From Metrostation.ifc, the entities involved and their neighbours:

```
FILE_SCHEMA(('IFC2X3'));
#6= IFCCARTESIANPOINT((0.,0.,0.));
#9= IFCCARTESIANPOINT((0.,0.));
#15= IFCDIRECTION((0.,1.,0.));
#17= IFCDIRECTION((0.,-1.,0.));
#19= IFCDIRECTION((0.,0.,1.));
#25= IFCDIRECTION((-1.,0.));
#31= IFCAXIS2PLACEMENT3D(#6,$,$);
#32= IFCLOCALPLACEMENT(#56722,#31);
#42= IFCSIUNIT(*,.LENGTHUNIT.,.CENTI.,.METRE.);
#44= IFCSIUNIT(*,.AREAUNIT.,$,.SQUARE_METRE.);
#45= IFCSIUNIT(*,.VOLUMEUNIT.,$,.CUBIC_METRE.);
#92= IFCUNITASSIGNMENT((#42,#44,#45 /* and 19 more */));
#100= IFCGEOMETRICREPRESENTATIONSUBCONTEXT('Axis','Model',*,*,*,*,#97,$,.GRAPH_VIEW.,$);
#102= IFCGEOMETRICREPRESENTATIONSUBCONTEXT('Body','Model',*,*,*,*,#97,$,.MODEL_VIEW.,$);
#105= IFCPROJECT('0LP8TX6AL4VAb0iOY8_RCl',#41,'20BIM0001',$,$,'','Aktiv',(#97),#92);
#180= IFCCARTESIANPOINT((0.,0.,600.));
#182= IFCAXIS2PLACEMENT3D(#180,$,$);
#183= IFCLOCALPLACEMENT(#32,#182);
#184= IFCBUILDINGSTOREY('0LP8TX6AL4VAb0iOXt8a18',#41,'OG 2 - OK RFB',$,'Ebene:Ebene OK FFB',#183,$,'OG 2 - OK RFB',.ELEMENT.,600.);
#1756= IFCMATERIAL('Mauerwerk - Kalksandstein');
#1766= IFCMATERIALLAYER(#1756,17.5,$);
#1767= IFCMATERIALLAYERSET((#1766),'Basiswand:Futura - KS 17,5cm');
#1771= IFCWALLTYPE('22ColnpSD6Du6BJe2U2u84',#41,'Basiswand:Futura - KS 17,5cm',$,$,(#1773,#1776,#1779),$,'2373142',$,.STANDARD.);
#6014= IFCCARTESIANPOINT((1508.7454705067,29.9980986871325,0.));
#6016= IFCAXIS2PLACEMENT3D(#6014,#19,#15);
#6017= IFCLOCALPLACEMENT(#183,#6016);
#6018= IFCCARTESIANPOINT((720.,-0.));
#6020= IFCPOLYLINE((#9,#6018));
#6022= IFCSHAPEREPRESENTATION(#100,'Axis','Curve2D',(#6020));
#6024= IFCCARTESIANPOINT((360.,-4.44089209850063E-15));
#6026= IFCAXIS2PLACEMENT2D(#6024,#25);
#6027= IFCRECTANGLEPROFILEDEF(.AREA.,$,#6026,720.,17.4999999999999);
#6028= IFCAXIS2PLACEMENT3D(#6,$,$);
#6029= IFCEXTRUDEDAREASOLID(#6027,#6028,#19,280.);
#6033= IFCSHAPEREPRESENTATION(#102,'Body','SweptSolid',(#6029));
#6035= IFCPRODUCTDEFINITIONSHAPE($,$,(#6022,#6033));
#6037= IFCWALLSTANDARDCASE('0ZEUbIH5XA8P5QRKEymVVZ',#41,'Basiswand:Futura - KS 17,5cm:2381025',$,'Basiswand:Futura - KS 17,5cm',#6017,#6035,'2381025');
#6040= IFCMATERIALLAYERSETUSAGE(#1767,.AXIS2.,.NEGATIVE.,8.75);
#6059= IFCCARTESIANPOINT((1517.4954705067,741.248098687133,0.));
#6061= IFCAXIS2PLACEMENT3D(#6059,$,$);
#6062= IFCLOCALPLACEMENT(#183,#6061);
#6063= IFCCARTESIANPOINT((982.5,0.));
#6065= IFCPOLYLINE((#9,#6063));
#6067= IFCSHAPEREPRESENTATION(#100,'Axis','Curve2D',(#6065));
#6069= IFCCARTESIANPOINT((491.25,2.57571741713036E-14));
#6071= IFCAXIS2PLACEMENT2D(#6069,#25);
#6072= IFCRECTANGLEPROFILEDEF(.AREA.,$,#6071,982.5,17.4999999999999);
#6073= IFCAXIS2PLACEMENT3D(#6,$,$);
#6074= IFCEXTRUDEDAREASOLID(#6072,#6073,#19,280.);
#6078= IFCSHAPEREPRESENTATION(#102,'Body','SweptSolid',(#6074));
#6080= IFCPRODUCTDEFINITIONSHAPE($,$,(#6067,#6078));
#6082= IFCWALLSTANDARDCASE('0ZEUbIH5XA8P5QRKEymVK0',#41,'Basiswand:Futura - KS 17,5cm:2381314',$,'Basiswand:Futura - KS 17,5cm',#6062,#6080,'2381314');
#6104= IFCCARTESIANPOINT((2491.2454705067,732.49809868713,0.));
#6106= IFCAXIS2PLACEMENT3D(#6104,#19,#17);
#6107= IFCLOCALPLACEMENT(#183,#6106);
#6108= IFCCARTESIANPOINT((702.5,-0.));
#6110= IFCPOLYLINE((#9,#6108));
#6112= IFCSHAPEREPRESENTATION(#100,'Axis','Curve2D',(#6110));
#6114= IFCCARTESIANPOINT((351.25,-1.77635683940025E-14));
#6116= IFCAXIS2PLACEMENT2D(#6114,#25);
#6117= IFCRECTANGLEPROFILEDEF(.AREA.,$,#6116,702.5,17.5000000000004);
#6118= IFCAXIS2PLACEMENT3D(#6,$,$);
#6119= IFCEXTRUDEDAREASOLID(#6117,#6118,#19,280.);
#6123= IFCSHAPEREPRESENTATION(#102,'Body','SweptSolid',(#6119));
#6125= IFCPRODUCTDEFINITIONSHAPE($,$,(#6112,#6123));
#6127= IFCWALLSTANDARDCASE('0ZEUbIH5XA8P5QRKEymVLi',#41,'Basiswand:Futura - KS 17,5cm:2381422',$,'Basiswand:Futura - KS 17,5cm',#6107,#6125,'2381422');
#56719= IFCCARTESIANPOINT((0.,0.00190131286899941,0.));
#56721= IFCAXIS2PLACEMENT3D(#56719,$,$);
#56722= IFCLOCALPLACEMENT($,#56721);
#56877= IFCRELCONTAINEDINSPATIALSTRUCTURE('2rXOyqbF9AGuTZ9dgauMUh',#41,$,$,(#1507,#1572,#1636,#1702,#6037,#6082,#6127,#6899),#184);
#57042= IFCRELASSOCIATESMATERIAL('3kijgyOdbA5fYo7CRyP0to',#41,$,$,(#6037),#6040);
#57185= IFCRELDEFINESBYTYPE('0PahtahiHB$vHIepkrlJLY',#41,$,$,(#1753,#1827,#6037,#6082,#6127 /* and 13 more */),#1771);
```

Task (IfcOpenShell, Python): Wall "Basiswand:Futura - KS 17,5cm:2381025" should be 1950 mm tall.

```python
import ifcopenshell
import ifcopenshell.geom
import ifcopenshell.util.representation
import ifcopenshell.util.shape
import ifcopenshell.util.unit

model = ifcopenshell.open("Metrostation.ifc")
unit_scale = ifcopenshell.util.unit.calculate_unit_scale(model)
settings = ifcopenshell.geom.settings()


def volume(element):
    """Net volume in cubic metres, openings subtracted."""
    shape = ifcopenshell.geom.create_shape(settings, element)
    return ifcopenshell.util.shape.get_volume(shape.geometry)


wall = model.by_guid("0ZEUbIH5XA8P5QRKEymVVZ")
before = volume(wall)

body = ifcopenshell.util.representation.get_representation(wall, "Model", "Body")
solid = body.Items[0]
old_height = solid.Depth
solid.Depth = 1.95 / unit_scale
after = volume(wall)

print(f"height {old_height:g} -> {solid.Depth:g}, volume {before:.3f} -> {after:.3f} m3")

model.write("Metrostation_updated.ifc")
```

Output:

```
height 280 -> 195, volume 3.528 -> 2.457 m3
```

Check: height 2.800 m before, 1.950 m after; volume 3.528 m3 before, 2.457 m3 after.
